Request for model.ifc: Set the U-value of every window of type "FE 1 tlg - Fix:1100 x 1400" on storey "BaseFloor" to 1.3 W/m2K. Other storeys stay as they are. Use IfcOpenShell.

First a look at what the model holds.

```python
import ifcopenshell
import ifcopenshell.util.element

model = ifcopenshell.open("model.ifc")
print(model.schema)
storey = next(s for s in model.by_type("IfcBuildingStorey") if s.Name == "BaseFloor")
windows = [e for e in ifcopenshell.util.element.get_decomposition(storey) if e.is_a("IfcWindow")]
seen = {}
for e in windows:
    element_type = ifcopenshell.util.element.get_type(e)
    key = (element_type.Name if element_type != e and element_type else None, ifcopenshell.util.element.get_pset(e, "Pset_WindowCommon", "ThermalTransmittance"))
    seen[key] = seen.get(key, 0) + 1
for (name, value), count in sorted(seen.items(), key=str):
    print(count, "x", name, "|", value)
```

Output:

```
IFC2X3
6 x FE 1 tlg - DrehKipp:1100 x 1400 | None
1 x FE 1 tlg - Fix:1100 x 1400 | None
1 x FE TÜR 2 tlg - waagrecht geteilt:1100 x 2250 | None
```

```python
import ifcopenshell
import ifcopenshell.api.pset
import ifcopenshell.util.element

model = ifcopenshell.open("model.ifc")

storey = next(s for s in model.by_type("IfcBuildingStorey") if s.Name == "BaseFloor")
windows = [e for e in ifcopenshell.util.element.get_decomposition(storey) if e.is_a("IfcWindow")]

count = 0
for e in windows:
    element_type = ifcopenshell.util.element.get_type(e)
    if element_type in (None, e) or element_type.Name != "FE 1 tlg - Fix:1100 x 1400":
        continue
    # add_pset returns the element's existing set when there is one.
    pset = ifcopenshell.api.pset.add_pset(model, product=e, name="Pset_WindowCommon")
    ifcopenshell.api.pset.edit_pset(model, pset=pset, properties={"ThermalTransmittance": 1.3})
    count += 1

print(count, "windows updated")

model.write("model_rev.ifc")
```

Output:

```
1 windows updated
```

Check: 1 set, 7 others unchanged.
